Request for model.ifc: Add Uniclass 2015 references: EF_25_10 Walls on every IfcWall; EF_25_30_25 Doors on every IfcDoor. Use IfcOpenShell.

First a look at what the model holds.

```python
import ifcopenshell

model = ifcopenshell.open("model.ifc")
print(model.schema)
print("classifications:", [c.Name for c in model.by_type("IfcClassification")])
for ifc_class in ("IfcDoor", "IfcRoof", "IfcStair", "IfcWall", "IfcWindow"):
    print(ifc_class, len(model.by_type(ifc_class)))
```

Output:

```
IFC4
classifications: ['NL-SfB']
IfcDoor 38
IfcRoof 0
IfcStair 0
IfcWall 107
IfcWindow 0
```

```python
import ifcopenshell
import ifcopenshell.api.classification

model = ifcopenshell.open("model.ifc")

system = ifcopenshell.api.classification.add_classification(model, classification="Uniclass 2015")

codes = {
    "IfcWall": ("EF_25_10", "Walls"),
    "IfcDoor": ("EF_25_30_25", "Doors"),
}
for ifc_class, (code, name) in codes.items():
    products = model.by_type(ifc_class)
    ifcopenshell.api.classification.add_reference(
        model, products=products, classification=system, identification=code, name=name
    )
    print(code, len(products))

model.write("model_edited.ifc")
```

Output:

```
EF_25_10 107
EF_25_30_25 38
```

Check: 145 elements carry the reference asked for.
